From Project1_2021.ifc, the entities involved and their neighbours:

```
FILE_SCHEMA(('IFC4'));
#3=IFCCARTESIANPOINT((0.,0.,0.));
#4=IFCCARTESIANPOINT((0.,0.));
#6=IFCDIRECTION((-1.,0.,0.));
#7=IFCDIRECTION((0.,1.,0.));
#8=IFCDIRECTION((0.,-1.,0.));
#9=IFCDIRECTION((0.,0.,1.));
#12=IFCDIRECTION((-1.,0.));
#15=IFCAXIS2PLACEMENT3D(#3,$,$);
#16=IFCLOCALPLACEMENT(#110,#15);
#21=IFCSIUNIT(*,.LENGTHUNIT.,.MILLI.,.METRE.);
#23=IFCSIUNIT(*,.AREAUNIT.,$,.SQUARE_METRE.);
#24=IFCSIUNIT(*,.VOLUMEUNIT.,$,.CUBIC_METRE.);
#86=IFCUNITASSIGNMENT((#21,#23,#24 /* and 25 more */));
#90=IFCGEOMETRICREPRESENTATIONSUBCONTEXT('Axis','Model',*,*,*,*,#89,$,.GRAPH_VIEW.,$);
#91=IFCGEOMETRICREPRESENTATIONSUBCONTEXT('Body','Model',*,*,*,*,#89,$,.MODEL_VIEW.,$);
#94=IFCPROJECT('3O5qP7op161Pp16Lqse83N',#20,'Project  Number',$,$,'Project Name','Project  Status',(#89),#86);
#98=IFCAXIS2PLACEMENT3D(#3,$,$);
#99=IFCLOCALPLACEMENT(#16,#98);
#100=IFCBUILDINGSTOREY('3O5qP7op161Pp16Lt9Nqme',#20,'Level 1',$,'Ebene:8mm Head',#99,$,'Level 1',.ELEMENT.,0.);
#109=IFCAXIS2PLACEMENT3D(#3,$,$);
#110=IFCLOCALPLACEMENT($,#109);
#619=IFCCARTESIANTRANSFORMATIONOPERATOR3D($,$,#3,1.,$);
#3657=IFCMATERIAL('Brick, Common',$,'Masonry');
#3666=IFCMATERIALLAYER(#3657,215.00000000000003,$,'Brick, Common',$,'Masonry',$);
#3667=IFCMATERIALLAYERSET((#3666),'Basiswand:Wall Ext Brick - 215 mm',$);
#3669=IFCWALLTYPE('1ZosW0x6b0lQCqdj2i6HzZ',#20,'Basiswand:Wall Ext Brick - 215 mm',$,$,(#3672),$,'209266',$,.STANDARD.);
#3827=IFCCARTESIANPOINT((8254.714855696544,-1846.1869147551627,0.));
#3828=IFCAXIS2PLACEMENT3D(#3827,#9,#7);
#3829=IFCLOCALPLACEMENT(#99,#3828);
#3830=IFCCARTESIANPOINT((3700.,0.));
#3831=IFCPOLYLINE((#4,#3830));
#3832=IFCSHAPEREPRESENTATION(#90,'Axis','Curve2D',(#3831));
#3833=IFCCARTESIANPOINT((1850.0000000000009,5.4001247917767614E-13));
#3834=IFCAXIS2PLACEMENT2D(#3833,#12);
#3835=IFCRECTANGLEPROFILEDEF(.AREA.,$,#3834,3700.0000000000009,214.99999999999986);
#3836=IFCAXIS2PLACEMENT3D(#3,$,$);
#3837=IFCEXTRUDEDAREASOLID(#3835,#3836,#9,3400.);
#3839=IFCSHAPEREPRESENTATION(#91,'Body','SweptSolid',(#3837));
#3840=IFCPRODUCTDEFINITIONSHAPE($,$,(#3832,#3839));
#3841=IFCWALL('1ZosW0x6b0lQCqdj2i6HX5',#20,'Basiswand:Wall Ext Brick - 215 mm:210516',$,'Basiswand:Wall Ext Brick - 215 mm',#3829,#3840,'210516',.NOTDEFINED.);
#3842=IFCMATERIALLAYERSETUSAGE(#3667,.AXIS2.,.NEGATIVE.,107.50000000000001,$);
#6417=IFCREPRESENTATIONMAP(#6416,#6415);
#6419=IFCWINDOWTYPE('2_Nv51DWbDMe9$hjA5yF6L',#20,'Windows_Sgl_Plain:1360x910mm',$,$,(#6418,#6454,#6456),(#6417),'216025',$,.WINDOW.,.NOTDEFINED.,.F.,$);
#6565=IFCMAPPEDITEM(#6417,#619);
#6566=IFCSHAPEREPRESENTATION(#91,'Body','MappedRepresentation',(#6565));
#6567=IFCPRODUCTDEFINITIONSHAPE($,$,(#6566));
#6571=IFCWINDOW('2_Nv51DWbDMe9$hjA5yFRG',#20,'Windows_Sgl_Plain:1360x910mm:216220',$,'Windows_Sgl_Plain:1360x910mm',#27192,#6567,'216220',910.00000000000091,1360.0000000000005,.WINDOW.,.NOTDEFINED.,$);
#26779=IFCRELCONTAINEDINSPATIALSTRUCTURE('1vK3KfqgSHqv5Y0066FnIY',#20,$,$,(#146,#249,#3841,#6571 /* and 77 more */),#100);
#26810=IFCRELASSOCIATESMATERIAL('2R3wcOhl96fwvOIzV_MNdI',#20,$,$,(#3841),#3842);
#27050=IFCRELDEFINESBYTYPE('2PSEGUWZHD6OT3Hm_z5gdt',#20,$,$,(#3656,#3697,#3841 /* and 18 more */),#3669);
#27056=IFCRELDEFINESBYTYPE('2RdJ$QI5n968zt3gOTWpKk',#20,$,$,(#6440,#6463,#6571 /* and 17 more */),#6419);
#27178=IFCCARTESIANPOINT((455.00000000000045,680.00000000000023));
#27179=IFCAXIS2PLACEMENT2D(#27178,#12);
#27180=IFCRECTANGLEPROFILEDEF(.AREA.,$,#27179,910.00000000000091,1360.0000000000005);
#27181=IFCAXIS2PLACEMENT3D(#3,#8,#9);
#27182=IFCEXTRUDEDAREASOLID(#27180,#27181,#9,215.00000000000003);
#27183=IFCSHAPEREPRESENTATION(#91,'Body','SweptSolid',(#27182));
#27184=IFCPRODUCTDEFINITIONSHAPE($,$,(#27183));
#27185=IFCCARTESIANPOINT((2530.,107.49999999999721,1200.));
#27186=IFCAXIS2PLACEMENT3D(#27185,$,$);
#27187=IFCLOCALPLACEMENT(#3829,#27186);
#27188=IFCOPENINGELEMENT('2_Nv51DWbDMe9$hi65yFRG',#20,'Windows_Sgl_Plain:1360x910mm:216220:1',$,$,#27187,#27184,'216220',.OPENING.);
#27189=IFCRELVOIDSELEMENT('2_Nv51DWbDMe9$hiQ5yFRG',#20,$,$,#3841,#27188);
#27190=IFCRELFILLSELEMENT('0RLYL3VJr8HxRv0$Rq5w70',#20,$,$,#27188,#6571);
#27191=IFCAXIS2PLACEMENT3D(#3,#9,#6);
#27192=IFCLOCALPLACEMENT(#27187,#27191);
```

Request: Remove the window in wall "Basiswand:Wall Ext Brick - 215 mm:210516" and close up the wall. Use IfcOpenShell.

```python
import ifcopenshell
import ifcopenshell.api.feature
import ifcopenshell.api.root
import ifcopenshell.geom
import ifcopenshell.util.shape

model = ifcopenshell.open("Project1_2021.ifc")
settings = ifcopenshell.geom.settings()


def volume(element):
    """Net volume in cubic metres, openings subtracted."""
    shape = ifcopenshell.geom.create_shape(settings, element)
    return ifcopenshell.util.shape.get_volume(shape.geometry)


window = model.by_id(6571)
opening = window.FillsVoids[0].RelatingOpeningElement
wall = opening.VoidsElements[0].RelatingBuildingElement
before = volume(wall)

ifcopenshell.api.root.remove_product(model, product=window)
ifcopenshell.api.feature.remove_feature(model, feature=opening)

after = volume(wall)

print(f"wall volume {before:.3f} -> {after:.3f} m3")

model.write("Project1_2021-out.ifc")
```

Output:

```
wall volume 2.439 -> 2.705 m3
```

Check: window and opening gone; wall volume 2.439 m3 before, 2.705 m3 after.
